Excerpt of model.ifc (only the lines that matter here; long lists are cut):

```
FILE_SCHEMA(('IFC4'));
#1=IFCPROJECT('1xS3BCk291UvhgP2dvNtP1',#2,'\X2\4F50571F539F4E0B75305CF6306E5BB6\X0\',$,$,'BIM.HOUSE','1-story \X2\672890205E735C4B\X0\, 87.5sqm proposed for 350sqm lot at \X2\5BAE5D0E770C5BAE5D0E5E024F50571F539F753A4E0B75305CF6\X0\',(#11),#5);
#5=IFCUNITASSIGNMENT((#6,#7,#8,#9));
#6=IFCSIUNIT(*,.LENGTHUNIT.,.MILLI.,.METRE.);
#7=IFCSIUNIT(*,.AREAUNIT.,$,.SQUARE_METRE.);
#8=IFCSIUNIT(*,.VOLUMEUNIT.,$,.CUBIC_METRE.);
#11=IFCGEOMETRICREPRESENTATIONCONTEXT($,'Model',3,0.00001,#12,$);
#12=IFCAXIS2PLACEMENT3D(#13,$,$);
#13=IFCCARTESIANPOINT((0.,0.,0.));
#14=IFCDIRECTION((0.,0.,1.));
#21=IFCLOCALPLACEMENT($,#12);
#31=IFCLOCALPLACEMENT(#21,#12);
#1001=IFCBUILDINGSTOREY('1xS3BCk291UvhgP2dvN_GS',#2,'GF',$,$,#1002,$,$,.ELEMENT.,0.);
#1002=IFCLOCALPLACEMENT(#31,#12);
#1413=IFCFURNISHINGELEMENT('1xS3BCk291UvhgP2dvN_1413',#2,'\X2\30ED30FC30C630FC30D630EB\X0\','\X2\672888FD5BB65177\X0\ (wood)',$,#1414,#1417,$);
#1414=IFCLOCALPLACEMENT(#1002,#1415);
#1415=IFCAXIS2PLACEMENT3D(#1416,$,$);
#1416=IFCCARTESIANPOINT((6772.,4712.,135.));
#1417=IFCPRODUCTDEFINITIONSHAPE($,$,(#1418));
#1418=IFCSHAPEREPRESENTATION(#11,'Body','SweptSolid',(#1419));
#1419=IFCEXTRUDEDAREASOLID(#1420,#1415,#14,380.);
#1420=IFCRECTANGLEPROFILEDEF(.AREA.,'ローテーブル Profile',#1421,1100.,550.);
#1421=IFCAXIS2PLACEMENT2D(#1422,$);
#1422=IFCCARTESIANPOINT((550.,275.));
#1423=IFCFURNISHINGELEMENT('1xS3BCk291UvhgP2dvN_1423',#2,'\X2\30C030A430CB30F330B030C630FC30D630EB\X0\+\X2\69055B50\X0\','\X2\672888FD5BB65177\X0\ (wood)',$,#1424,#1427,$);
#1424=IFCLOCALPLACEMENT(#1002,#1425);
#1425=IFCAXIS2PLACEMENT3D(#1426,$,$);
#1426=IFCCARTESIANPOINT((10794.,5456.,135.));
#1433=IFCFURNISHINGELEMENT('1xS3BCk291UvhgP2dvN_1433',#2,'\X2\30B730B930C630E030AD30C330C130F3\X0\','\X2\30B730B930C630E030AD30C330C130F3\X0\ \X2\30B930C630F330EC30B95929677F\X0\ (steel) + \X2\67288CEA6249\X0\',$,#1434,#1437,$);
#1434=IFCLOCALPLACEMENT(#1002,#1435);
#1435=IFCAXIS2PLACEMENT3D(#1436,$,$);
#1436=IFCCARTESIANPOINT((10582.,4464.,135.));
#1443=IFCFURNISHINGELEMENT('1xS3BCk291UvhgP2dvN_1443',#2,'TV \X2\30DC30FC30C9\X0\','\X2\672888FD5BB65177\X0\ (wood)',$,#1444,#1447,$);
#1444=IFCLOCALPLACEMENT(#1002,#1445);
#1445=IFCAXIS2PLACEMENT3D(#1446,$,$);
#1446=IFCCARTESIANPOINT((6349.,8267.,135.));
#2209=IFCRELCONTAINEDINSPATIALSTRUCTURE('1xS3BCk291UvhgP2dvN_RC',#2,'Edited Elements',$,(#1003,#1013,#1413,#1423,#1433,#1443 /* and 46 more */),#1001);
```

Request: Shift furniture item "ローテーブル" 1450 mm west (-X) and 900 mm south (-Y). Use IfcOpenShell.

```python
import ifcopenshell
import ifcopenshell.api.geometry
import ifcopenshell.util.placement

model = ifcopenshell.open("model.ifc")

item = model.by_guid("1xS3BCk291UvhgP2dvN_1413")
matrix = ifcopenshell.util.placement.get_local_placement(item.ObjectPlacement)
matrix[0, 3] -= 1450.0
matrix[1, 3] -= 900.0
ifcopenshell.api.geometry.edit_object_placement(model, product=item, matrix=matrix, is_si=False)

print(ifcopenshell.util.placement.get_local_placement(item.ObjectPlacement).round(3) + 0.0)

model.write("model_edited.ifc")
```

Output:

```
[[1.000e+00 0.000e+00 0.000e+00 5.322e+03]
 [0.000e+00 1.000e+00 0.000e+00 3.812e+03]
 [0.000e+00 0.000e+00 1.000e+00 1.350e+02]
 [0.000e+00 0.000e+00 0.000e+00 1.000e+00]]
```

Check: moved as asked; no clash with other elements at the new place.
